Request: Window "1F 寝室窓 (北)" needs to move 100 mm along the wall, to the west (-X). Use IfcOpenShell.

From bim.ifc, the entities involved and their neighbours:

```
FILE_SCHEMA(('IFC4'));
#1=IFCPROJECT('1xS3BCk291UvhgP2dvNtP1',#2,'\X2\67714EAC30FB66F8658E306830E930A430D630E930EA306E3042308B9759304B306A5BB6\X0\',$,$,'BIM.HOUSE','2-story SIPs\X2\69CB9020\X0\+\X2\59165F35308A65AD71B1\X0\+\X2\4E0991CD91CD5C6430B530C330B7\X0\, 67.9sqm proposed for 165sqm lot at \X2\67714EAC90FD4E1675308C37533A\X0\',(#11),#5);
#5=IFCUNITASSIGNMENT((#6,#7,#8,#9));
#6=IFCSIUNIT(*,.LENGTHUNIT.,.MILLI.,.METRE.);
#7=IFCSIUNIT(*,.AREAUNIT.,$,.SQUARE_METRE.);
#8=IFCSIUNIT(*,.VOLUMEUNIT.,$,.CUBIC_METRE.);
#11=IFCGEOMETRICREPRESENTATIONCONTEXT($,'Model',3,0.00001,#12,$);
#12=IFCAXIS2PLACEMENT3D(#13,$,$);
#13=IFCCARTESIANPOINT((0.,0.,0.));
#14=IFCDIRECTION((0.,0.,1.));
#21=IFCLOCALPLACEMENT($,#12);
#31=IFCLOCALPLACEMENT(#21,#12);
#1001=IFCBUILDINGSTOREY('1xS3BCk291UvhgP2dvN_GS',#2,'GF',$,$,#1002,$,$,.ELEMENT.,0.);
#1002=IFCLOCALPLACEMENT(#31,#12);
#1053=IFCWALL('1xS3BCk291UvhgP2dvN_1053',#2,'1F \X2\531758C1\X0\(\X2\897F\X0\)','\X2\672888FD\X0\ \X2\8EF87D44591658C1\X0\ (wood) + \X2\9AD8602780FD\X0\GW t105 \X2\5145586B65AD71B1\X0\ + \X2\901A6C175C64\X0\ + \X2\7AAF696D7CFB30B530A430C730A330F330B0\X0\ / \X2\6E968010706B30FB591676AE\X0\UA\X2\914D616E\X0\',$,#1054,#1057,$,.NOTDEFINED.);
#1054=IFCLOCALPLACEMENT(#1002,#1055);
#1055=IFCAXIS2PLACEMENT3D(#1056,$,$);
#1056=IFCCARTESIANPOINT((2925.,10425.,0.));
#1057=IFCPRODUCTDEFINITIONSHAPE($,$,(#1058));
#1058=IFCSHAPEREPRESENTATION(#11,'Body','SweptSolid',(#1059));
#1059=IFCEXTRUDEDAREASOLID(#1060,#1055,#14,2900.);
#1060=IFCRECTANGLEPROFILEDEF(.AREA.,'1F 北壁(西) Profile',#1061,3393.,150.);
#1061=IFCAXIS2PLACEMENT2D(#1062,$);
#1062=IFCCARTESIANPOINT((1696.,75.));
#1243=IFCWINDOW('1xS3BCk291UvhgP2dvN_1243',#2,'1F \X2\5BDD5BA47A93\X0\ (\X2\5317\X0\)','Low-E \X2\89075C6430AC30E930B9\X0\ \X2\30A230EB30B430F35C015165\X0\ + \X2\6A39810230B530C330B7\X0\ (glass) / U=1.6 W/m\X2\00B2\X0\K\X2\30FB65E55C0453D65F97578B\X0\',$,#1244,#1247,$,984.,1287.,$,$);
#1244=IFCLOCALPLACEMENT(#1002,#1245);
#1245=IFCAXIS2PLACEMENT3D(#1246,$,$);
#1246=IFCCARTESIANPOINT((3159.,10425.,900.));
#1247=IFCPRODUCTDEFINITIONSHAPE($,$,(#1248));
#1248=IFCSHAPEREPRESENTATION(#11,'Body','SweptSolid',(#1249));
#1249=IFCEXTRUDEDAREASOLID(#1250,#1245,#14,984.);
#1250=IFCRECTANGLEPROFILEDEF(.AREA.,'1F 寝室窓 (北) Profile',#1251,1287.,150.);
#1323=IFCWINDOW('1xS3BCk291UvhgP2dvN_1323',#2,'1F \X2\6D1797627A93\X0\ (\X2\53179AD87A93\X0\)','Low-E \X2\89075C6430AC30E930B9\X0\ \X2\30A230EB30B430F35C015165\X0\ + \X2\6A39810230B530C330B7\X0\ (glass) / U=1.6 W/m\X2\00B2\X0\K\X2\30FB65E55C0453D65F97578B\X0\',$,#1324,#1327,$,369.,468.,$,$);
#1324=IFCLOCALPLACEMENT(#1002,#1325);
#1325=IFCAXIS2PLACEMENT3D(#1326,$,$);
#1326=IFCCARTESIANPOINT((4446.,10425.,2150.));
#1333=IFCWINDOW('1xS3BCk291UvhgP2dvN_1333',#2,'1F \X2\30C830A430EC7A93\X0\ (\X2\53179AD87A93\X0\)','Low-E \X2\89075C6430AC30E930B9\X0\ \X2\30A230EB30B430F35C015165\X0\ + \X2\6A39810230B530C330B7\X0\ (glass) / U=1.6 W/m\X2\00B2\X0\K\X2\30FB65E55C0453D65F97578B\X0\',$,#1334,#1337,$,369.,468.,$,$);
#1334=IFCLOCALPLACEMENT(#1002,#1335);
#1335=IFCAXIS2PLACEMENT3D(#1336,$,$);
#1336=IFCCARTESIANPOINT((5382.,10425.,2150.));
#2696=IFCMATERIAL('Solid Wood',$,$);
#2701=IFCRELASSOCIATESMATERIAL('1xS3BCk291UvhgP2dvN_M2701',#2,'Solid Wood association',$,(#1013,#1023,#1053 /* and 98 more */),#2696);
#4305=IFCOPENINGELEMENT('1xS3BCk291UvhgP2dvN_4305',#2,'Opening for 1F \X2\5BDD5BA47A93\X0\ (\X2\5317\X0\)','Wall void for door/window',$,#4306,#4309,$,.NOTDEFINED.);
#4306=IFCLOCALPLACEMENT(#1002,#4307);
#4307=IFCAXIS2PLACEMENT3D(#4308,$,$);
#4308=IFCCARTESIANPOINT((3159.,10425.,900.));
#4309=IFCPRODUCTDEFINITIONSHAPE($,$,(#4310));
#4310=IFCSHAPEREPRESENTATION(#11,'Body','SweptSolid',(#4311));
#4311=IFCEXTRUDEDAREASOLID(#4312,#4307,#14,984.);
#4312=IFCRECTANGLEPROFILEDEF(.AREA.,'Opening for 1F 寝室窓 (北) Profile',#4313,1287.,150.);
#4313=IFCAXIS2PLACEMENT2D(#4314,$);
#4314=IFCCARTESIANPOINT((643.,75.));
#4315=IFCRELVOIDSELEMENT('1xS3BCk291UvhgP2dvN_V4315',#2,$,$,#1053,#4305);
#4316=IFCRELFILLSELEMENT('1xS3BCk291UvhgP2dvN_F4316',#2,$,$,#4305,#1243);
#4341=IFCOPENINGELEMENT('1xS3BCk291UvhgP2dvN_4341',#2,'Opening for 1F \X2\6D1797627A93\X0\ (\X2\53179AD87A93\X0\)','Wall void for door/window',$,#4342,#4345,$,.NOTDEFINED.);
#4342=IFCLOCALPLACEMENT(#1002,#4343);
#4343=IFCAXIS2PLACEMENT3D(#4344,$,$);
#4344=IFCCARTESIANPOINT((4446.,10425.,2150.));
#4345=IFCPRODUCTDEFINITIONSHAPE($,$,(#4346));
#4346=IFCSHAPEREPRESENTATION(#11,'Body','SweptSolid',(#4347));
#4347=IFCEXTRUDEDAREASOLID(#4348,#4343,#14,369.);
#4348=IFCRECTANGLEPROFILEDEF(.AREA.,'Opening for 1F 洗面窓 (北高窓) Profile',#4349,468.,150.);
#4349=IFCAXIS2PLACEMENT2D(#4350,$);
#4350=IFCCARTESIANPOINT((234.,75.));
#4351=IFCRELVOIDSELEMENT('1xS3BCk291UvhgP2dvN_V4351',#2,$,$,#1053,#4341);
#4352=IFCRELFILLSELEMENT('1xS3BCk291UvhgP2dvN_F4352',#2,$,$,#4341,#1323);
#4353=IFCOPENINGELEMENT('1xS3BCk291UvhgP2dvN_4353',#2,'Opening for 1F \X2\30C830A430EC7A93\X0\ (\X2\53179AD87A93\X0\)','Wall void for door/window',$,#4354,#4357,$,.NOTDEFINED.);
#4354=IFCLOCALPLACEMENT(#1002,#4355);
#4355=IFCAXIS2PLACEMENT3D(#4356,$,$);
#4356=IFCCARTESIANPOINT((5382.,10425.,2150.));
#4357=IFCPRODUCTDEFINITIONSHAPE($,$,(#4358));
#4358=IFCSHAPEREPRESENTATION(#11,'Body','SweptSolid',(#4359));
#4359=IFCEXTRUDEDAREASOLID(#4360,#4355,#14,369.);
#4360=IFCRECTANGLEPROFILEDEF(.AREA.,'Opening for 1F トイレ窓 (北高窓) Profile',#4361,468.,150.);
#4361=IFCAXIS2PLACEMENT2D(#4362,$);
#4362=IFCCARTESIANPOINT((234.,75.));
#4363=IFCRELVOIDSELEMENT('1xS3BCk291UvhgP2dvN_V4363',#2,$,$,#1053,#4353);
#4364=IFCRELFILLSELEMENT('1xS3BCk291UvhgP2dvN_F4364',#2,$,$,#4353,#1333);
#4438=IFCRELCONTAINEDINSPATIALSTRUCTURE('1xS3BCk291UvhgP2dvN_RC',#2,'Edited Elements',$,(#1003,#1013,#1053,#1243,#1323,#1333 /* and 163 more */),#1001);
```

```python
import ifcopenshell
import ifcopenshell.api.geometry
import ifcopenshell.util.placement

model = ifcopenshell.open("bim.ifc")

window = model.by_guid("1xS3BCk291UvhgP2dvN_1243")
opening = window.FillsVoids[0].RelatingOpeningElement
wall = opening.VoidsElements[0].RelatingBuildingElement

wall_matrix = ifcopenshell.util.placement.get_local_placement(wall.ObjectPlacement)
shift = wall_matrix[:3, 0] * -100.0
before = ifcopenshell.util.placement.get_local_placement(window.ObjectPlacement)[:3, 3].copy()

# The window is not placed relative to its opening, so move both.
for product in (opening, window):
    matrix = ifcopenshell.util.placement.get_local_placement(product.ObjectPlacement)
    matrix[:3, 3] += shift
    ifcopenshell.api.geometry.edit_object_placement(model, product=product, matrix=matrix, is_si=False)

after = ifcopenshell.util.placement.get_local_placement(window.ObjectPlacement)[:3, 3]
print("window moved by", (after - before).round(3) + 0.0)

model.write("bim_rev.ifc")
```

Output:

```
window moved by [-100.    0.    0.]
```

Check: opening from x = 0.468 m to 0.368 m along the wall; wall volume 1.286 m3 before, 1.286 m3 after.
